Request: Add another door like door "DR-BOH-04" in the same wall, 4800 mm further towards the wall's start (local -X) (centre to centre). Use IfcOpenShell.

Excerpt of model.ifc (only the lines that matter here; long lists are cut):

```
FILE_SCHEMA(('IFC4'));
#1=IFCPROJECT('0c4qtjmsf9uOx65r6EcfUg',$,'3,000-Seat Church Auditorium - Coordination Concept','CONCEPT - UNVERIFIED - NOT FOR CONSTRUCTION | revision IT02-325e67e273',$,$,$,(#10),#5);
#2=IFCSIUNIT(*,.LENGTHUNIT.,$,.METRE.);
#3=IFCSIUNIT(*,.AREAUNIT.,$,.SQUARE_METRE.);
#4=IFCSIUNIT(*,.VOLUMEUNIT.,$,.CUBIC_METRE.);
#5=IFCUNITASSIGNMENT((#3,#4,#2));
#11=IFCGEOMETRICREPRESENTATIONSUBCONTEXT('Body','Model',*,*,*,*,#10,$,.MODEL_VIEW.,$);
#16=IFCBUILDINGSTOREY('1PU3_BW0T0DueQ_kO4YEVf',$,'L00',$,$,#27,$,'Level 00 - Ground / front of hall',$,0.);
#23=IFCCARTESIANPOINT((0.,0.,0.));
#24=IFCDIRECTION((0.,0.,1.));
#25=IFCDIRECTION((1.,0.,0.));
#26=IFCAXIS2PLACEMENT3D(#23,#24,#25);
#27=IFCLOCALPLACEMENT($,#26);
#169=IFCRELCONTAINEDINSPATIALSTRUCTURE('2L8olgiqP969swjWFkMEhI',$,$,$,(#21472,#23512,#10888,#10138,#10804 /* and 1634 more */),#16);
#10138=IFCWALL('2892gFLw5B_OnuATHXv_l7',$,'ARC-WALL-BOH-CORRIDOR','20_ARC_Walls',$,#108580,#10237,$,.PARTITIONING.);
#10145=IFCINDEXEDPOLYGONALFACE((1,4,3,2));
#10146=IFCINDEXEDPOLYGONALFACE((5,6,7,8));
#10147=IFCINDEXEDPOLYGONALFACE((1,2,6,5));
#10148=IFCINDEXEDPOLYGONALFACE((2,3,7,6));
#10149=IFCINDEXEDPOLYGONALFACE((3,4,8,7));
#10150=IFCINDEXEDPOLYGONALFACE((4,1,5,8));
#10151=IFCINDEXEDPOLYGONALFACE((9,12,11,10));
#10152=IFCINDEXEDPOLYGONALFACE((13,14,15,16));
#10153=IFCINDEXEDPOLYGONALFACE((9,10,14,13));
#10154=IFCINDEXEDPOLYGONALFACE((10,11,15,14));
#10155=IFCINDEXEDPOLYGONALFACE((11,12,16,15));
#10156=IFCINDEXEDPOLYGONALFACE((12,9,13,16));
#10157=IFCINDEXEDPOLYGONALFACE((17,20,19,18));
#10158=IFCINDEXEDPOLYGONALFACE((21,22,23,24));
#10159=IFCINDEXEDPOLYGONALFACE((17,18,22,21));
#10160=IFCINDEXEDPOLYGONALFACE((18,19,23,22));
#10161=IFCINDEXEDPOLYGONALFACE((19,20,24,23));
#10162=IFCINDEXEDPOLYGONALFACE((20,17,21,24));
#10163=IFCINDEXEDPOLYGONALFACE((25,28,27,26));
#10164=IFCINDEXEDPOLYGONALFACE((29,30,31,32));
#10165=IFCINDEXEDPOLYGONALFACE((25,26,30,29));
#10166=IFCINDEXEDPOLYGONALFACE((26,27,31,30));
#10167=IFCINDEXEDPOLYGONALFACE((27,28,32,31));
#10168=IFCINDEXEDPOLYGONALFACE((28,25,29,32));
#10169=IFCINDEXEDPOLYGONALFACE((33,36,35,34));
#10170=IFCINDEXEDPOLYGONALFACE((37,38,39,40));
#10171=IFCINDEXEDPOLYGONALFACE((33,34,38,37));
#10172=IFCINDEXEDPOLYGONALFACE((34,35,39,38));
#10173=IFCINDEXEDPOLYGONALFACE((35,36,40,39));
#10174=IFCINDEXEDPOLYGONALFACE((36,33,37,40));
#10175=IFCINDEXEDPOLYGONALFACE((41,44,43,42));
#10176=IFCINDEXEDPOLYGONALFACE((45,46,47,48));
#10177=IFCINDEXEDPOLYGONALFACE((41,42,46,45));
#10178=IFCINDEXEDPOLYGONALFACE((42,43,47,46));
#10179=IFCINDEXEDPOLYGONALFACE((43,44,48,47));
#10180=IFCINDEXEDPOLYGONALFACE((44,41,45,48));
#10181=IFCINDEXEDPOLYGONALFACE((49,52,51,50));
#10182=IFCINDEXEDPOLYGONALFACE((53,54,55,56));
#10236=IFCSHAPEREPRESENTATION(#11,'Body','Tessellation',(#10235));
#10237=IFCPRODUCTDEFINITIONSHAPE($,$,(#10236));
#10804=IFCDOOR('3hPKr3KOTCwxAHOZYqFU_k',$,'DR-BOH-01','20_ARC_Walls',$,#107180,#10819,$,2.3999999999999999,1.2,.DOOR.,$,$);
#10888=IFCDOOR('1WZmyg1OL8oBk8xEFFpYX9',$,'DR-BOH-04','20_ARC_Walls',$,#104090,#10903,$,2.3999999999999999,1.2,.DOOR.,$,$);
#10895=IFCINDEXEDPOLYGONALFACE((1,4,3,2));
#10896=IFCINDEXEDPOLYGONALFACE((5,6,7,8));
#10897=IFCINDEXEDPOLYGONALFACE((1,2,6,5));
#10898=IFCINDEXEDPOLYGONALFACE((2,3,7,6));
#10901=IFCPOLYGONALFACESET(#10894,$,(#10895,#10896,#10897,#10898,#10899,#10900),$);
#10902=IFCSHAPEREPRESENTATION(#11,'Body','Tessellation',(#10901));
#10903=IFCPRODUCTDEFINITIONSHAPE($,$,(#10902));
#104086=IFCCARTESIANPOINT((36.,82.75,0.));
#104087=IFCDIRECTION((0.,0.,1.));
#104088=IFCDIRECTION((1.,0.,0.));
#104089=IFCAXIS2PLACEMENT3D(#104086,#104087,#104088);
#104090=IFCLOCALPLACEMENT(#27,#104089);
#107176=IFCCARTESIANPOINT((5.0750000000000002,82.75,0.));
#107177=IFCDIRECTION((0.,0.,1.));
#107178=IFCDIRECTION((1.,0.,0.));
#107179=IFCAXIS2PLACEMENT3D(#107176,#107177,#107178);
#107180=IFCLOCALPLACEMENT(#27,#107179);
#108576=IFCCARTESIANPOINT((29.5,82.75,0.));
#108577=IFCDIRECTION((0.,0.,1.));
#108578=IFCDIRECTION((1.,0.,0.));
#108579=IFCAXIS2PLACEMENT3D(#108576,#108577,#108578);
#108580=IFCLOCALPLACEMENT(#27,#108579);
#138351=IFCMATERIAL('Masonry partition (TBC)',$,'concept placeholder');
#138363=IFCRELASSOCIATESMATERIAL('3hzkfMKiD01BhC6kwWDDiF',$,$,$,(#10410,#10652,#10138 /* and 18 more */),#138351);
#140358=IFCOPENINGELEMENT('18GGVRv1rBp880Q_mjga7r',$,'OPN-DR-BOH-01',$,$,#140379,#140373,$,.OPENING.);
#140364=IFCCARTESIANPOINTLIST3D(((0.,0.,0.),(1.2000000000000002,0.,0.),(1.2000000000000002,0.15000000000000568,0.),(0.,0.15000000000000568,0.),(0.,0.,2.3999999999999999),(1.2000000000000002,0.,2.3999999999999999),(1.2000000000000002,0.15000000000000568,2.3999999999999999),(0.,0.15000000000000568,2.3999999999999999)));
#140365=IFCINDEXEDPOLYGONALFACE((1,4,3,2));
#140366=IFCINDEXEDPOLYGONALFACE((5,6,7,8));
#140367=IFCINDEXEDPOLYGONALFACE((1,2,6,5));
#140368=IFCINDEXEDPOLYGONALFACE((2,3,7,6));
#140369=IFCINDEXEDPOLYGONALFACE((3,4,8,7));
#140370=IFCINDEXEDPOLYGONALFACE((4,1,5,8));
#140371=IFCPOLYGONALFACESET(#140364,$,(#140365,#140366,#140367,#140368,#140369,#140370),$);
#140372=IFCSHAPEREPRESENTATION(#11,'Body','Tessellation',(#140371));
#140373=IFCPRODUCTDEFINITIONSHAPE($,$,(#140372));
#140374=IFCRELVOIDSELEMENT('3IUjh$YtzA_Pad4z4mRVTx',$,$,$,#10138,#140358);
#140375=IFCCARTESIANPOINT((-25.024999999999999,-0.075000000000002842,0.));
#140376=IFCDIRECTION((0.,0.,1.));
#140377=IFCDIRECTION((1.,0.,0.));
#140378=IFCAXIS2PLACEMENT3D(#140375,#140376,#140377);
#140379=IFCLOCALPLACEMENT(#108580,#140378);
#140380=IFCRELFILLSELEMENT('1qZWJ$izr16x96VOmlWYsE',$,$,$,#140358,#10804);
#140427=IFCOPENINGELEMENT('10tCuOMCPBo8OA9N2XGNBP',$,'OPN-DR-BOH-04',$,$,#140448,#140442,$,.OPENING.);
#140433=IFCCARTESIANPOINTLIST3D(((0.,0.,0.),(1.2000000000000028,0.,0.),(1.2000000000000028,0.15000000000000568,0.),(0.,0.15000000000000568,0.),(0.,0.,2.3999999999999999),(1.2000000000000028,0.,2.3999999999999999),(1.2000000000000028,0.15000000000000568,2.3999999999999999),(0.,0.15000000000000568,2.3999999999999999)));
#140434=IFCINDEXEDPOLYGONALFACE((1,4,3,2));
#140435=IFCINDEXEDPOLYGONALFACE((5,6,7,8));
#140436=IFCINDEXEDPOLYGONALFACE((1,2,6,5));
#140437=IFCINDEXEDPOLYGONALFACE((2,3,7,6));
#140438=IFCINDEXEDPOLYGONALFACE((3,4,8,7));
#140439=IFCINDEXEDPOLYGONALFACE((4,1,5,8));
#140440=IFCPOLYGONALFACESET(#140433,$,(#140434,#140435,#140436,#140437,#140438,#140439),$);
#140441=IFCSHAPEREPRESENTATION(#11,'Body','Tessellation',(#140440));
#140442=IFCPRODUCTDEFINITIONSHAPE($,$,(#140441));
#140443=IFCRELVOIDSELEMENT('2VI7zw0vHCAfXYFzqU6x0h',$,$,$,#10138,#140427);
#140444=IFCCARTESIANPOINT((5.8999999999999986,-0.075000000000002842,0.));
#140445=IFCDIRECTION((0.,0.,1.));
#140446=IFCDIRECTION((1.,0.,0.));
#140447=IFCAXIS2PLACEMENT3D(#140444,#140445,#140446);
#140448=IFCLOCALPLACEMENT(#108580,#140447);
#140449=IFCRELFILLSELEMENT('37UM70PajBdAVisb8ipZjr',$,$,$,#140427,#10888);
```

```python
import ifcopenshell
import ifcopenshell.api.feature
import ifcopenshell.api.geometry
import ifcopenshell.api.root
import ifcopenshell.geom
import ifcopenshell.util.element
import ifcopenshell.util.placement
import ifcopenshell.util.shape

model = ifcopenshell.open("model.ifc")
settings = ifcopenshell.geom.settings()


def volume(element):
    """Net volume in cubic metres, openings subtracted."""
    shape = ifcopenshell.geom.create_shape(settings, element)
    return ifcopenshell.util.shape.get_volume(shape.geometry)


door = model.by_guid("1WZmyg1OL8oBk8xEFFpYX9")
opening = door.FillsVoids[0].RelatingOpeningElement
wall = opening.VoidsElements[0].RelatingBuildingElement
before = volume(wall)
shift = ifcopenshell.util.placement.get_local_placement(wall.ObjectPlacement)[:3, 0] * -4.8

# copy_class copies the void relationship, type, container and properties, but no geometry.
new_opening = ifcopenshell.api.root.copy_class(model, product=opening)
new_opening.Representation = ifcopenshell.util.element.copy_deep(
    model, opening.Representation, exclude=["IfcGeometricRepresentationContext", "IfcRepresentationMap"]
)
new_door = ifcopenshell.api.root.copy_class(model, product=door)
new_door.Representation = ifcopenshell.util.element.copy_deep(
    model, door.Representation, exclude=["IfcGeometricRepresentationContext", "IfcRepresentationMap"]
)
ifcopenshell.api.feature.add_filling(model, opening=new_opening, element=new_door)

for old, new in ((opening, new_opening), (door, new_door)):
    matrix = ifcopenshell.util.placement.get_local_placement(old.ObjectPlacement)
    matrix[:3, 3] += shift
    ifcopenshell.api.geometry.edit_object_placement(model, product=new, matrix=matrix, is_si=False)

after = volume(wall)

print(f"wall volume {before:.3f} -> {after:.3f} m3")

model.write("model_rev.ifc")
```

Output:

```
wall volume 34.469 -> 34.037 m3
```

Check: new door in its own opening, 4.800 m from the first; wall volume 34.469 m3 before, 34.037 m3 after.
